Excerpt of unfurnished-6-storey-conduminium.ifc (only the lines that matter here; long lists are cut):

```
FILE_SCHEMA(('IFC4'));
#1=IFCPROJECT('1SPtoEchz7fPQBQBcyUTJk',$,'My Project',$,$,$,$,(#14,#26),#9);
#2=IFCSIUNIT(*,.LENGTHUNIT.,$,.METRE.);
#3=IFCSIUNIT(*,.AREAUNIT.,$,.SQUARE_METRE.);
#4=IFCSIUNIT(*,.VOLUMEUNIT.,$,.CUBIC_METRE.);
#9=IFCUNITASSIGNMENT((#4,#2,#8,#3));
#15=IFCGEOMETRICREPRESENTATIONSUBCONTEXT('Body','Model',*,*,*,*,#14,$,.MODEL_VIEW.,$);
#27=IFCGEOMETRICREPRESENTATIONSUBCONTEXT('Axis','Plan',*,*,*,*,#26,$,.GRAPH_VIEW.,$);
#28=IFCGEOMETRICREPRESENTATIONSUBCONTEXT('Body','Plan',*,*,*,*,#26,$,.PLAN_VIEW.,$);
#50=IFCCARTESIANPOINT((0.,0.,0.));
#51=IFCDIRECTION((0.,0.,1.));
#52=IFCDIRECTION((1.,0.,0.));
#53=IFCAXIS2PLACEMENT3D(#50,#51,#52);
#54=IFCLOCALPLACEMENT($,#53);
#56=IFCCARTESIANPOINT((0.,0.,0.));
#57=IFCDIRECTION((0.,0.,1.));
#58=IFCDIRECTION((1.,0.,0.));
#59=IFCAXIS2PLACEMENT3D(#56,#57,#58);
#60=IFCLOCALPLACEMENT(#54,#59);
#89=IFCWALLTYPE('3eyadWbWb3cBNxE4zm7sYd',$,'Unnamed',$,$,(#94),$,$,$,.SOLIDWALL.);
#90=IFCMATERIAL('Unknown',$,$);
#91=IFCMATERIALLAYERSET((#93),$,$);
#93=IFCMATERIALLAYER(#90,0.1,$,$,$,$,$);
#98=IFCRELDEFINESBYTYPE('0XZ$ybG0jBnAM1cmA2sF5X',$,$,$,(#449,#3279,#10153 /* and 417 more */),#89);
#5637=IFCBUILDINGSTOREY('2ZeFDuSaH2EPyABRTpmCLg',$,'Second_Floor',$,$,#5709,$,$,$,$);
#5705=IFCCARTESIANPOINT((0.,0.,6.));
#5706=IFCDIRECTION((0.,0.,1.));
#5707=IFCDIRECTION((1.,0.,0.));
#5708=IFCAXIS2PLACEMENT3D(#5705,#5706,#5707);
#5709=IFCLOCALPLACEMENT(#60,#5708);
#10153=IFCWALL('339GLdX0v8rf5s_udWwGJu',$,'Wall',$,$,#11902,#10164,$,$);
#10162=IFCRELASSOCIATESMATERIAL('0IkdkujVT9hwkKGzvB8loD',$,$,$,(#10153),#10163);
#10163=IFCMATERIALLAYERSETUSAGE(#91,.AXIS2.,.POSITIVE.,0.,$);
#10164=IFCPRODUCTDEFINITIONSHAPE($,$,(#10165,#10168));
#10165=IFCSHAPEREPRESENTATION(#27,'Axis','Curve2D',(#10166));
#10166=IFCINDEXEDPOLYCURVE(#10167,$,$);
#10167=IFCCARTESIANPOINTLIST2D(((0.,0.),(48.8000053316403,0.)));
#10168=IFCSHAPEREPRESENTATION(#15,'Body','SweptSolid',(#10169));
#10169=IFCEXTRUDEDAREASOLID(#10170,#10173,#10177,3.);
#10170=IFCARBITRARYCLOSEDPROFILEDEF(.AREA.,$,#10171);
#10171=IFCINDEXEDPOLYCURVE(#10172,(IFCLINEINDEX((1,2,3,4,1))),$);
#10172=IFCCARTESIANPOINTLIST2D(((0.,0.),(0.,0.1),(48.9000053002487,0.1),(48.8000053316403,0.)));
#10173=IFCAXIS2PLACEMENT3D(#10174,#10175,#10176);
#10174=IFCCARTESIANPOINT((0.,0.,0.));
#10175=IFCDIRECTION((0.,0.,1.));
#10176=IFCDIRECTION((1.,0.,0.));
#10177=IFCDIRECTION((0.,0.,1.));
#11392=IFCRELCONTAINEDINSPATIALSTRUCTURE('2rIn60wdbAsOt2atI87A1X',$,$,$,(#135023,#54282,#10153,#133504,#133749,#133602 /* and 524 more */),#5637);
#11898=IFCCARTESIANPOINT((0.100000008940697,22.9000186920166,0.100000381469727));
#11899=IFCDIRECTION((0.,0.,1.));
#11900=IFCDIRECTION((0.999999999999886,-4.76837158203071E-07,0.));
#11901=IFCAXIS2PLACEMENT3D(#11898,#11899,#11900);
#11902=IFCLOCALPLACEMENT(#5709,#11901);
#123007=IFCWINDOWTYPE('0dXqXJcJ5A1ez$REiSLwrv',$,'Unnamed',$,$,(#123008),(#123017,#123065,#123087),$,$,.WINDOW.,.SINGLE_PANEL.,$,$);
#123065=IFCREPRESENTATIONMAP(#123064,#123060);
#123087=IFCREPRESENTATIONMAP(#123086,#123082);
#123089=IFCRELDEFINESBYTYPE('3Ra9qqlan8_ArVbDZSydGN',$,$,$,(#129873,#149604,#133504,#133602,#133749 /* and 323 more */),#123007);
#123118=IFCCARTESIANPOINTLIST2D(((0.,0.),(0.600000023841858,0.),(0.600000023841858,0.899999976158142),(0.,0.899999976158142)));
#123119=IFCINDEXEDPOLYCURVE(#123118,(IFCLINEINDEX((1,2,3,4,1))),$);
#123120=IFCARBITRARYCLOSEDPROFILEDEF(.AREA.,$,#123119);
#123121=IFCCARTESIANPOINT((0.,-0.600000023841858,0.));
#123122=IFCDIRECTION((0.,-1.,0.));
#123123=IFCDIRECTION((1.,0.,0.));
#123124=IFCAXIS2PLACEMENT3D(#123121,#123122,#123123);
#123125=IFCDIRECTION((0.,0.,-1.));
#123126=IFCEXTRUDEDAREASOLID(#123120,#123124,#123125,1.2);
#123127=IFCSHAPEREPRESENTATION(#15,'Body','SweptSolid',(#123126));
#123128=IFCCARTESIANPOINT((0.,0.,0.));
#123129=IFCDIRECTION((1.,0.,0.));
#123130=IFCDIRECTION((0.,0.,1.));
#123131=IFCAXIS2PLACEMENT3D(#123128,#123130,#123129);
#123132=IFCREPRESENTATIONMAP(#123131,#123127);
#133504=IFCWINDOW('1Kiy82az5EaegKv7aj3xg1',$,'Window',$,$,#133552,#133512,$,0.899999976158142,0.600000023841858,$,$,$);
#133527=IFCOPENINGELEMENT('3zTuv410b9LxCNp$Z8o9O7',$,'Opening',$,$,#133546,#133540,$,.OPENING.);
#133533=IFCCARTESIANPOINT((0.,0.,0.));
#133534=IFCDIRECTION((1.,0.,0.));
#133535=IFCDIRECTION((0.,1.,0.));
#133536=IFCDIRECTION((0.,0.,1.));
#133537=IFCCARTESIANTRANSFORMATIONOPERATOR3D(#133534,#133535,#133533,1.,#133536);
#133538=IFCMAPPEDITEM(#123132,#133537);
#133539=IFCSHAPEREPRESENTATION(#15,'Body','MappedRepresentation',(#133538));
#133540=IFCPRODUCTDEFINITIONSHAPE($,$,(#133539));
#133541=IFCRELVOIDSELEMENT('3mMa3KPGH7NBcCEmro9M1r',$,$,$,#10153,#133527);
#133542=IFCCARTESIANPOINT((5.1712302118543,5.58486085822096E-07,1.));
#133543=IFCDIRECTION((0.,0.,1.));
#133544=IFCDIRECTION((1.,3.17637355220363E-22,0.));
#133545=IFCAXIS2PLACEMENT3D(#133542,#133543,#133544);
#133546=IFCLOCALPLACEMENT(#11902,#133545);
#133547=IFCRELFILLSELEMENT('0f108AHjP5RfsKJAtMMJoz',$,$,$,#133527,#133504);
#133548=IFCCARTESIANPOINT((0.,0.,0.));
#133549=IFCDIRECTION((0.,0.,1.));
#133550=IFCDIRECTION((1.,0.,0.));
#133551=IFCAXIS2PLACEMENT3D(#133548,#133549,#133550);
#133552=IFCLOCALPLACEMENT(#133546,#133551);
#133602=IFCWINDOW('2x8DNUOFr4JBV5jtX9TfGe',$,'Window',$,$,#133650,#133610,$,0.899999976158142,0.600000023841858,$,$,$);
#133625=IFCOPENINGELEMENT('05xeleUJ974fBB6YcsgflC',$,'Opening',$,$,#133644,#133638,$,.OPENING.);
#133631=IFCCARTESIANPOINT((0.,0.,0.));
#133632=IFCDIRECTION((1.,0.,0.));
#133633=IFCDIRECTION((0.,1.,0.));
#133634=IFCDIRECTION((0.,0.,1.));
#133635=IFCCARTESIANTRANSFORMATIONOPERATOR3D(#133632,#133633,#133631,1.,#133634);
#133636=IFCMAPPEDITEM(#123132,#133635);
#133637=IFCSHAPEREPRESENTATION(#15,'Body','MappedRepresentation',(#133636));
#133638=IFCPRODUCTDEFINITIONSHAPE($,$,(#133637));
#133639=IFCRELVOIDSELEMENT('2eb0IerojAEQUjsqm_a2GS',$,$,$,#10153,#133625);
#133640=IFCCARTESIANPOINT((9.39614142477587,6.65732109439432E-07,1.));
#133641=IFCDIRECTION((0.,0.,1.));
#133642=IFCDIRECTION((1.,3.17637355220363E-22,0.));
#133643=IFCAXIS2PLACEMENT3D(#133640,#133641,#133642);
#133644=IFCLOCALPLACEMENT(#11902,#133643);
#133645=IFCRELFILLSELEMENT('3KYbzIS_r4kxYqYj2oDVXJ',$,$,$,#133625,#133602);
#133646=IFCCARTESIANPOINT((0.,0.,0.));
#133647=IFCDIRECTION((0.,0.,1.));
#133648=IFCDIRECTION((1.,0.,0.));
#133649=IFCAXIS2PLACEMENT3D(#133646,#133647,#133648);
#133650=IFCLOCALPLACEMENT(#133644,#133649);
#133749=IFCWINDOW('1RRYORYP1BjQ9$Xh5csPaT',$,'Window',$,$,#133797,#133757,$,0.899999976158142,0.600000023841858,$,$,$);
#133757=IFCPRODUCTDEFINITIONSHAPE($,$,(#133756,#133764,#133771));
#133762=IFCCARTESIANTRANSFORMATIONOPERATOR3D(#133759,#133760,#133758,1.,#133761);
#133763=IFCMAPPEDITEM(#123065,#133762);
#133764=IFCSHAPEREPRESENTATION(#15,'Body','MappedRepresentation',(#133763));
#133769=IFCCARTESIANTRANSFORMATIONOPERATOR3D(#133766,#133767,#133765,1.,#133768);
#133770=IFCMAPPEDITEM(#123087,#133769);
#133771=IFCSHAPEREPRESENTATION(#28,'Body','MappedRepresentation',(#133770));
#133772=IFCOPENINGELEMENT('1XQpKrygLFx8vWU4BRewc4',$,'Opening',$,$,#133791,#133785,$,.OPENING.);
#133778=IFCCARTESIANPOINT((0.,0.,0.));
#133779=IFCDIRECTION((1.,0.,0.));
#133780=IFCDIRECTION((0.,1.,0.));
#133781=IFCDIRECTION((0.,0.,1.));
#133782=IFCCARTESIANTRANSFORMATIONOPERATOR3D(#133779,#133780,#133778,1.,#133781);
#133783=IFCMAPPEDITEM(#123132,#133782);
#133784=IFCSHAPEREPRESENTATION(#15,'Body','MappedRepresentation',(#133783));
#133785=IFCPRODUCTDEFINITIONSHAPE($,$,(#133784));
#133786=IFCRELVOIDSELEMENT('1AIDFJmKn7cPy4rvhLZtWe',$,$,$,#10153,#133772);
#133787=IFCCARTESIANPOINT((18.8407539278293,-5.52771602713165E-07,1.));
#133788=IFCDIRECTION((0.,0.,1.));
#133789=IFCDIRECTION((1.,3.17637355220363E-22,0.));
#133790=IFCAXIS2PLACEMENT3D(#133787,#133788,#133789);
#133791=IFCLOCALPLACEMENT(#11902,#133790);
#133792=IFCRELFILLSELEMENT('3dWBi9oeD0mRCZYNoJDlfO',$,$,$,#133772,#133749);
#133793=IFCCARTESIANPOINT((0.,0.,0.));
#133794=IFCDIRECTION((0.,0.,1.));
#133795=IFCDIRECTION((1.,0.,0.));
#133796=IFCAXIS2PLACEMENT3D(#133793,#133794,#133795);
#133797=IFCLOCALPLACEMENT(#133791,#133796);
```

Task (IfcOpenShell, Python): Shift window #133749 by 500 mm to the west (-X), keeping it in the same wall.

```python
import ifcopenshell
import ifcopenshell.api.geometry
import ifcopenshell.util.placement
import ifcopenshell.util.unit

model = ifcopenshell.open("unfurnished-6-storey-conduminium.ifc")
unit_scale = ifcopenshell.util.unit.calculate_unit_scale(model)

window = model.by_id(133749)
opening = window.FillsVoids[0].RelatingOpeningElement
wall = opening.VoidsElements[0].RelatingBuildingElement

wall_matrix = ifcopenshell.util.placement.get_local_placement(wall.ObjectPlacement)
shift = wall_matrix[:3, 0] * -0.5 / unit_scale
before = ifcopenshell.util.placement.get_local_placement(window.ObjectPlacement)[:3, 3].copy()

# The window is placed relative to its opening, so it follows when the opening moves.
matrix = ifcopenshell.util.placement.get_local_placement(opening.ObjectPlacement)
matrix[:3, 3] += shift
ifcopenshell.api.geometry.edit_object_placement(
    model, product=opening, matrix=matrix, is_si=False, should_transform_children=True
)

after = ifcopenshell.util.placement.get_local_placement(window.ObjectPlacement)[:3, 3]
print("window moved by", (after - before).round(3) + 0.0)

model.write("unfurnished-6-storey-conduminium_updated.ifc")
```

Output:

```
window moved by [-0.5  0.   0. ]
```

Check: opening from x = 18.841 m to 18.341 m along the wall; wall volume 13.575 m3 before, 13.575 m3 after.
